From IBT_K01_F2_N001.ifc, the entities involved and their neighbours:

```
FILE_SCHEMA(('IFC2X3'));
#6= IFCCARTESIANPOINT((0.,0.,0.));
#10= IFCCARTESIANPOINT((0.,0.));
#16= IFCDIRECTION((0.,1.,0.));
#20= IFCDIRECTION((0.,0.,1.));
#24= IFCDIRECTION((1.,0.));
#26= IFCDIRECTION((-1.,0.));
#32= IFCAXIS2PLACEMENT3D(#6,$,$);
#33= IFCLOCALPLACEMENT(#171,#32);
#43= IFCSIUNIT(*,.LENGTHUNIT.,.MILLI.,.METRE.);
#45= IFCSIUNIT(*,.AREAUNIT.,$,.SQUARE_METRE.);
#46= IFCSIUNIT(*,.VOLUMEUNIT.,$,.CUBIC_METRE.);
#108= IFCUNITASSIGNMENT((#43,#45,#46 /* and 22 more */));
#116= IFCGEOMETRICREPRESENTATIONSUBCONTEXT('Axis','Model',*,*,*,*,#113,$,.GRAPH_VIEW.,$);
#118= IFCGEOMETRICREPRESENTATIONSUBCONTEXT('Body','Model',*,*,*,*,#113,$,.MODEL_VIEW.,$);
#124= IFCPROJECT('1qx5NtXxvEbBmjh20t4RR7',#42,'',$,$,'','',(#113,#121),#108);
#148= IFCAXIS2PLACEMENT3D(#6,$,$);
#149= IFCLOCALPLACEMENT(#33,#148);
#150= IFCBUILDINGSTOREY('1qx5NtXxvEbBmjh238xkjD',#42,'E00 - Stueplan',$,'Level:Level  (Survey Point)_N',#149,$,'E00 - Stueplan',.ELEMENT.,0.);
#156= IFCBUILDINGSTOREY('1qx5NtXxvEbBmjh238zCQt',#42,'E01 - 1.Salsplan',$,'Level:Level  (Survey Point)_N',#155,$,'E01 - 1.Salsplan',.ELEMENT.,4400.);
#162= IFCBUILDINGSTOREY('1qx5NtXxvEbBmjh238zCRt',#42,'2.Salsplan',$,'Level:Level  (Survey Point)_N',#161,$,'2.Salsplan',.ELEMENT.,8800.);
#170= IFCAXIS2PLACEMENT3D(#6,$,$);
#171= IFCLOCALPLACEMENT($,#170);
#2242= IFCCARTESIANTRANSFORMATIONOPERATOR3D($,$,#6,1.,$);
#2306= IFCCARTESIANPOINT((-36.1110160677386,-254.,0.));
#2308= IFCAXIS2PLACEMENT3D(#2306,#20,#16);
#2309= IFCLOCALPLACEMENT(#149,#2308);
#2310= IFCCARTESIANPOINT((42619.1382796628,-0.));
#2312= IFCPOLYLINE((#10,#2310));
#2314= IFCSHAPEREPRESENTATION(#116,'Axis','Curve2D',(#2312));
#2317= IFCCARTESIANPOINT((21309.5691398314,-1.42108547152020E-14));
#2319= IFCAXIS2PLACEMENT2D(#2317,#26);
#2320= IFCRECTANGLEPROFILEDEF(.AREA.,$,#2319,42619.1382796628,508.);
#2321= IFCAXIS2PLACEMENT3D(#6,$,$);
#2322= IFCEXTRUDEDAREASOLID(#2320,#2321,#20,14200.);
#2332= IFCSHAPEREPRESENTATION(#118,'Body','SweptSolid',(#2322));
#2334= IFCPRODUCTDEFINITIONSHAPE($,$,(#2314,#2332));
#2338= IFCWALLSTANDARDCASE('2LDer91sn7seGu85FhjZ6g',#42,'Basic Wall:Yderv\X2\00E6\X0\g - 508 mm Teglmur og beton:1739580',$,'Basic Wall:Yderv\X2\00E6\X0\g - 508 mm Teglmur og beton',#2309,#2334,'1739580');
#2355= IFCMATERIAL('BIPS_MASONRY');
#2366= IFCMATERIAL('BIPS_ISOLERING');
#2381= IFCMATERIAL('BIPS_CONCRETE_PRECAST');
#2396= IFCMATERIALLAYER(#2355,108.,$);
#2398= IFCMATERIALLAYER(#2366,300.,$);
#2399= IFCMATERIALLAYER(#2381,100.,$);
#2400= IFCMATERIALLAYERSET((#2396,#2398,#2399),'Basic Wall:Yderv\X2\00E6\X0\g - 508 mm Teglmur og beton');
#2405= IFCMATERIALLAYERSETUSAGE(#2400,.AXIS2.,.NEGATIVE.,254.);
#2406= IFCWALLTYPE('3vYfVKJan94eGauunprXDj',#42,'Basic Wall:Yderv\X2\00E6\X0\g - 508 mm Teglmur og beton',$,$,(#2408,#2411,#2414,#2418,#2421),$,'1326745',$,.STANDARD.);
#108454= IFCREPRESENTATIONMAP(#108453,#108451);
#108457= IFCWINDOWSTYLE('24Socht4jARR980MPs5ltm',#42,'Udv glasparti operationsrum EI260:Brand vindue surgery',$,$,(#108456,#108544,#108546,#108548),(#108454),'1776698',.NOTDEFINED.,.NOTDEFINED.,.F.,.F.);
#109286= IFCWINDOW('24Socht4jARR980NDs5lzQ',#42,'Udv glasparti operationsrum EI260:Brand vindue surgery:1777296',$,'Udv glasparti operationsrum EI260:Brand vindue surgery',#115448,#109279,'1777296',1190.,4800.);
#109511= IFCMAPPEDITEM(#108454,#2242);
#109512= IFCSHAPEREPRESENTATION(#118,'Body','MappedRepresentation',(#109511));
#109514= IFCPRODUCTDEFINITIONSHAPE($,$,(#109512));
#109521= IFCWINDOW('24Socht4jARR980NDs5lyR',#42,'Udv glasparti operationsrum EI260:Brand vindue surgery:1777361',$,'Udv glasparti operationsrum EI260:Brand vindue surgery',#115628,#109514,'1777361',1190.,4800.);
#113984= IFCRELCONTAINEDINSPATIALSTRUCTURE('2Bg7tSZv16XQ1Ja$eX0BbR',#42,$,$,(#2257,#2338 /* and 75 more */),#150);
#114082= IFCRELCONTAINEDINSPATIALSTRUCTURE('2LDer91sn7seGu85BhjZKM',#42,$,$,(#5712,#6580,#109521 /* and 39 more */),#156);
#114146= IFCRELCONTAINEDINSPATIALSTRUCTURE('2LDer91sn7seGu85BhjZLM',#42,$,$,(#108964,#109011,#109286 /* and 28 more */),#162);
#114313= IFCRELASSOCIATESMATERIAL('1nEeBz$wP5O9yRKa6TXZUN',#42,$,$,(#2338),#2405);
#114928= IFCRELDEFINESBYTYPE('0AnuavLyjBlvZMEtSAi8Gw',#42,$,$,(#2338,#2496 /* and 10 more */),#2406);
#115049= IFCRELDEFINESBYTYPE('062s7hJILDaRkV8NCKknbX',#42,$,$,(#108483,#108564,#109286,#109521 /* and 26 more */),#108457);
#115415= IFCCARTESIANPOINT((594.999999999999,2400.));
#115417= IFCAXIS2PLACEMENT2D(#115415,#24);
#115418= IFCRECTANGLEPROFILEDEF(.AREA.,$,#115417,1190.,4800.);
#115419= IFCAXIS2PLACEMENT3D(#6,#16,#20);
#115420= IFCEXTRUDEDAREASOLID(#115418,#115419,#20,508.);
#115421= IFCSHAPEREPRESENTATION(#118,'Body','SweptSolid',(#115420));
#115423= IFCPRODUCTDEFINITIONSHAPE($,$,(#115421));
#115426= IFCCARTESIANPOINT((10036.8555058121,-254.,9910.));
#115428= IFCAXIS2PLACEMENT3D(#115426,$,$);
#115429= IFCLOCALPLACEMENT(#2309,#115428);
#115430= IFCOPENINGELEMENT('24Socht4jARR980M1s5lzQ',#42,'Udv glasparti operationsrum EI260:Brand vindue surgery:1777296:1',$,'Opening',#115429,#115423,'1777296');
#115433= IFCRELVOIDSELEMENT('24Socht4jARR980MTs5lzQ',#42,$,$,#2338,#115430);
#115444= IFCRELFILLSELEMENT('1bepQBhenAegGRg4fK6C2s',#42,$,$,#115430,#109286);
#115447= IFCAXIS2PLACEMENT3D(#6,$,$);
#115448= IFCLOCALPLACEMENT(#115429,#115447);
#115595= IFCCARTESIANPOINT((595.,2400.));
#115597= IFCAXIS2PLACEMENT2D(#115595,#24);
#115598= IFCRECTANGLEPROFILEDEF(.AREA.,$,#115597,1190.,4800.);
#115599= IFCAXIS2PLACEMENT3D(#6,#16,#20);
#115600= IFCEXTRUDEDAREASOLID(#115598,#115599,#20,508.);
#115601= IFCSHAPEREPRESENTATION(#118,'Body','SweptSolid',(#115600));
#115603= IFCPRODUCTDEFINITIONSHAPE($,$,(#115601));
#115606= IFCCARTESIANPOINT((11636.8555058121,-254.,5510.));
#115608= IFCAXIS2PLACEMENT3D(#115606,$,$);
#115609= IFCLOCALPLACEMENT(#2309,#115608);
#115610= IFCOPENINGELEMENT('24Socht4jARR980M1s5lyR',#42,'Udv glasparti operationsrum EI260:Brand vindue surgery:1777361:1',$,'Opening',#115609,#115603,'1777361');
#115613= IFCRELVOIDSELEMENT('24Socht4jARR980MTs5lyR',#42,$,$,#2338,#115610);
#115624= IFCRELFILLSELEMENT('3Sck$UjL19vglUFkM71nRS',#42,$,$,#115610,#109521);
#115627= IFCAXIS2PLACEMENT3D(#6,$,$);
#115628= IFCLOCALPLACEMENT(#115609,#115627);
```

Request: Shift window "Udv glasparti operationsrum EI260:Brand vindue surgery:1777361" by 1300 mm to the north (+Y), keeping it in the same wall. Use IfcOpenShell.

```python
import ifcopenshell
import ifcopenshell.api.geometry
import ifcopenshell.util.placement

model = ifcopenshell.open("IBT_K01_F2_N001.ifc")

window = model.by_id(109521)
opening = window.FillsVoids[0].RelatingOpeningElement
wall = opening.VoidsElements[0].RelatingBuildingElement

wall_matrix = ifcopenshell.util.placement.get_local_placement(wall.ObjectPlacement)
shift = wall_matrix[:3, 0] * 1300.0
before = ifcopenshell.util.placement.get_local_placement(window.ObjectPlacement)[:3, 3].copy()

# The window is placed relative to its opening, so it follows when the opening moves.
matrix = ifcopenshell.util.placement.get_local_placement(opening.ObjectPlacement)
matrix[:3, 3] += shift
ifcopenshell.api.geometry.edit_object_placement(
    model, product=opening, matrix=matrix, is_si=False, should_transform_children=True
)

after = ifcopenshell.util.placement.get_local_placement(window.ObjectPlacement)[:3, 3]
print("window moved by", (after - before).round(3) + 0.0)

model.write("IBT_K01_F2_N001_edited.ifc")
```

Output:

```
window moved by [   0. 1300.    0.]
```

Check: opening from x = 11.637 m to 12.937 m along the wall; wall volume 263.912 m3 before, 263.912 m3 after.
